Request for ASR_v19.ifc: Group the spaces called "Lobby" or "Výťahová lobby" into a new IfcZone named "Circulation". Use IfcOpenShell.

First a look at what the model holds.

```python
import ifcopenshell

model = ifcopenshell.open("ASR_v19.ifc")
print(model.schema)
seen = {}
for space in model.by_type("IfcSpace"):
    seen[space.LongName] = seen.get(space.LongName, 0) + 1
for name, count in sorted(seen.items(), key=str):
    print(count, "x", name)
print("zones:", [z.Name for z in model.by_type("IfcZone")][:20])
```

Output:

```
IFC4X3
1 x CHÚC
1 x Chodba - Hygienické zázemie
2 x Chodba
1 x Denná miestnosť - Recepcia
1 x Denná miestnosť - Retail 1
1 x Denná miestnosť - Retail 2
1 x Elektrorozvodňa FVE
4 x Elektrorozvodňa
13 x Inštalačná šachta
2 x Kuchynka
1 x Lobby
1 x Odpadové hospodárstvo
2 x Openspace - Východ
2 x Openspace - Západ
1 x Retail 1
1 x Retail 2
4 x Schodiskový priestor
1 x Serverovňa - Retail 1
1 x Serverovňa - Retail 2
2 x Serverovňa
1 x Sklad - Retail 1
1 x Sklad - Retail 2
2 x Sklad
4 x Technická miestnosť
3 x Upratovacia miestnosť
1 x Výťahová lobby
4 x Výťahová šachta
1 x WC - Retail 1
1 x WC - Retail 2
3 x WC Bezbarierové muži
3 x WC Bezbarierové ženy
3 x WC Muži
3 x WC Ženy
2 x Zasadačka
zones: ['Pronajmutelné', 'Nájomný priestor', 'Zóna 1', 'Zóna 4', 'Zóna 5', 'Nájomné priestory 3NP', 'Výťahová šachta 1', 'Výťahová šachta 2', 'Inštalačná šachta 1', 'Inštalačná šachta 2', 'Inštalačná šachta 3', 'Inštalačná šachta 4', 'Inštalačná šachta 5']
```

```python
import ifcopenshell
import ifcopenshell.api.group
import ifcopenshell.api.root

model = ifcopenshell.open("ASR_v19.ifc")

names = {"Lobby", "Výťahová lobby"}
spaces = [s for s in model.by_type("IfcSpace") if s.LongName in names]

zone = ifcopenshell.api.root.create_entity(model, ifc_class="IfcZone", name="Circulation")
ifcopenshell.api.group.assign_group(model, products=spaces, group=zone)
print(len(spaces), "spaces in", zone.Name)

model.write("ASR_v19_rev.ifc")
```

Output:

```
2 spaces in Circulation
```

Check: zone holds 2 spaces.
